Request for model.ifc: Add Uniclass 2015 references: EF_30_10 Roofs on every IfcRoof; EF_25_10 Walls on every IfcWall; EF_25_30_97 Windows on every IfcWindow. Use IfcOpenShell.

First a look at what the model holds.

```python
import ifcopenshell

model = ifcopenshell.open("model.ifc")
print(model.schema)
print("classifications:", [c.Name for c in model.by_type("IfcClassification")])
for ifc_class in ("IfcDoor", "IfcRoof", "IfcStair", "IfcWall", "IfcWindow"):
    print(ifc_class, len(model.by_type(ifc_class)))
```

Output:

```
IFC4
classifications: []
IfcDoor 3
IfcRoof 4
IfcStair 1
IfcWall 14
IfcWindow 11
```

```python
import ifcopenshell
import ifcopenshell.api.classification

model = ifcopenshell.open("model.ifc")

system = ifcopenshell.api.classification.add_classification(model, classification="Uniclass 2015")

codes = {
    "IfcRoof": ("EF_30_10", "Roofs"),
    "IfcWall": ("EF_25_10", "Walls"),
    "IfcWindow": ("EF_25_30_97", "Windows"),
}
for ifc_class, (code, name) in codes.items():
    products = model.by_type(ifc_class)
    ifcopenshell.api.classification.add_reference(
        model, products=products, classification=system, identification=code, name=name
    )
    print(code, len(products))

model.write("model_edited.ifc")
```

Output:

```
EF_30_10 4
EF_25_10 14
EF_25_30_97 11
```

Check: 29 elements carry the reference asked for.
